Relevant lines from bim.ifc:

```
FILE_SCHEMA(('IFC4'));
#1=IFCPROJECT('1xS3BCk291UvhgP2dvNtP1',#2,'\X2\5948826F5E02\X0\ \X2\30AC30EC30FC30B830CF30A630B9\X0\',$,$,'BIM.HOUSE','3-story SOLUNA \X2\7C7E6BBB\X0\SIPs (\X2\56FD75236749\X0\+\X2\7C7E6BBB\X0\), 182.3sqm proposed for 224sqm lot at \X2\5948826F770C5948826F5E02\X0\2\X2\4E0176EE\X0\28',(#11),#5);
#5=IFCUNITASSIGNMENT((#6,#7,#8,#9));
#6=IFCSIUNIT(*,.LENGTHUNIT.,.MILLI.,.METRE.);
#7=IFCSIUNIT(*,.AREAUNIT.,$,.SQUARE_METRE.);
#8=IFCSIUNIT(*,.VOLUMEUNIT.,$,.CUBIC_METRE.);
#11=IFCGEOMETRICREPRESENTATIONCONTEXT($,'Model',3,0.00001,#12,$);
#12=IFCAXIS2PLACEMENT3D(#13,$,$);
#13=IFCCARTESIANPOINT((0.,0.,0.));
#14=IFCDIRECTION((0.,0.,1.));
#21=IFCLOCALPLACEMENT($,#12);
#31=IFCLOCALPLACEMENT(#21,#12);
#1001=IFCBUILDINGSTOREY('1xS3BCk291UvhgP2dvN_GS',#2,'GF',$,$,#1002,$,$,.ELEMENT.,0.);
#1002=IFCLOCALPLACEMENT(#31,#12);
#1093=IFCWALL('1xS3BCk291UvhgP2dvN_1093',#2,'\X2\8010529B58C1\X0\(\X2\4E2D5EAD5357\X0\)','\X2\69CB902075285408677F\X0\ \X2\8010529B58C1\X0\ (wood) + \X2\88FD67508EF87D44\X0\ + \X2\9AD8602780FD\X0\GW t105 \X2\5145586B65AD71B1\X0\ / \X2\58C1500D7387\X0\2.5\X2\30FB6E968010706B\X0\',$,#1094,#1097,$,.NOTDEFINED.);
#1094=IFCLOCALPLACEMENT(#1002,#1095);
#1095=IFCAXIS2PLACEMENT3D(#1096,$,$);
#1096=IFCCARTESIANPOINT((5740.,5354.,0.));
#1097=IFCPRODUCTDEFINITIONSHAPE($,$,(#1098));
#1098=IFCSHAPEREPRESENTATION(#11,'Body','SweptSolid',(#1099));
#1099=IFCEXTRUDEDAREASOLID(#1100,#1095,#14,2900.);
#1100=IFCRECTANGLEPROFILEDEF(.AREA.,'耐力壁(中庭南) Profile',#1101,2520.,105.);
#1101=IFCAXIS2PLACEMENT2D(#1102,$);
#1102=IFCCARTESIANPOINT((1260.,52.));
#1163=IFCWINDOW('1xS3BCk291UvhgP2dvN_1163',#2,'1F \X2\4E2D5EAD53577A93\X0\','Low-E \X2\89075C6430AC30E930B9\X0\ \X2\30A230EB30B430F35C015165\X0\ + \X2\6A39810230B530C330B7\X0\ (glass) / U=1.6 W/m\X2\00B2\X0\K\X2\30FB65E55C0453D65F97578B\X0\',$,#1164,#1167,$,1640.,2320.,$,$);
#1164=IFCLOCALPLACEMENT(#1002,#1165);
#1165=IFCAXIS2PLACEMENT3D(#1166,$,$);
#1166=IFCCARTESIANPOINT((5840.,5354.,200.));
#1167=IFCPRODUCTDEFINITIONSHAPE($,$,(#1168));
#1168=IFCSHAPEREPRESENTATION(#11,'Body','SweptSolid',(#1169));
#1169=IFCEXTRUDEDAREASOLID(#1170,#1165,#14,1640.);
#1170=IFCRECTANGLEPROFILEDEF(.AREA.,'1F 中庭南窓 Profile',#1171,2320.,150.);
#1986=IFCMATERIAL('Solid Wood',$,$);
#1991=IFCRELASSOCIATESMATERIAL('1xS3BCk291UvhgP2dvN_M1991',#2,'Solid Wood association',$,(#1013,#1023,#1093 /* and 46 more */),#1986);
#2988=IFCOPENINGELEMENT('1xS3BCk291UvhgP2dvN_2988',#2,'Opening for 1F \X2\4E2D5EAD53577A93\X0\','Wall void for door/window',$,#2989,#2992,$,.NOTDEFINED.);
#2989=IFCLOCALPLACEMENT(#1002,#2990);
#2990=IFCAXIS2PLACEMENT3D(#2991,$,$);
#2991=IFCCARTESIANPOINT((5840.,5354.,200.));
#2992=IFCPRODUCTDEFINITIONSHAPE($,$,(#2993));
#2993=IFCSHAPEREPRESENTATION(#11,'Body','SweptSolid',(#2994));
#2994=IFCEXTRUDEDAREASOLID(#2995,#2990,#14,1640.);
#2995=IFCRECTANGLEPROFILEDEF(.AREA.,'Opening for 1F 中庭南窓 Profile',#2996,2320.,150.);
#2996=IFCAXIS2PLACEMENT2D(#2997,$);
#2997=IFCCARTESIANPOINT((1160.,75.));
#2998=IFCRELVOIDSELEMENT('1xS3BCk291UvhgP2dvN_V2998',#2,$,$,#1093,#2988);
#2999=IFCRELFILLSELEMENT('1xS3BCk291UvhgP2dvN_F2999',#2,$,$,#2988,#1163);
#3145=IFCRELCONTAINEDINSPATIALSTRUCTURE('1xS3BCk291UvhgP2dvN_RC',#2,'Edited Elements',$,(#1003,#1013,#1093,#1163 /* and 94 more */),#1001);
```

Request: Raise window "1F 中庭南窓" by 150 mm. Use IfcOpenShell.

```python
import numpy as np
import ifcopenshell
import ifcopenshell.api.geometry
import ifcopenshell.util.placement
import ifcopenshell.util.unit

model = ifcopenshell.open("bim.ifc")
unit_scale = ifcopenshell.util.unit.calculate_unit_scale(model)

window = model.by_guid("1xS3BCk291UvhgP2dvN_1163")
opening = window.FillsVoids[0].RelatingOpeningElement
dz = 150.0

shift = np.array([0.0, 0.0, dz])
# The window is not placed relative to its opening, so move both.
for product in (opening, window):
    matrix = ifcopenshell.util.placement.get_local_placement(product.ObjectPlacement)
    matrix[:3, 3] += shift
    ifcopenshell.api.geometry.edit_object_placement(model, product=product, matrix=matrix, is_si=False)

print(f"moved by {dz * unit_scale:+.3f} m")

model.write("bim_v2.ifc")
```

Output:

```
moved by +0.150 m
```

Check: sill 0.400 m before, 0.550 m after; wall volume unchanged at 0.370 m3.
